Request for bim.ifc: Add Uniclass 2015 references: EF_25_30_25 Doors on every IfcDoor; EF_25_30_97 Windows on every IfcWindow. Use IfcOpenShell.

First a look at what the model holds.

```python
import ifcopenshell

model = ifcopenshell.open("bim.ifc")
print(model.schema)
print("classifications:", [c.Name for c in model.by_type("IfcClassification")])
for ifc_class in ("IfcDoor", "IfcRoof", "IfcStair", "IfcWall", "IfcWindow"):
    print(ifc_class, len(model.by_type(ifc_class)))
```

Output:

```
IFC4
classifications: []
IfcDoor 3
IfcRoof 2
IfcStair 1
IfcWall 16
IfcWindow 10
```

```python
import ifcopenshell
import ifcopenshell.api.classification

model = ifcopenshell.open("bim.ifc")

system = ifcopenshell.api.classification.add_classification(model, classification="Uniclass 2015")

codes = {
    "IfcDoor": ("EF_25_30_25", "Doors"),
    "IfcWindow": ("EF_25_30_97", "Windows"),
}
for ifc_class, (code, name) in codes.items():
    products = model.by_type(ifc_class)
    ifcopenshell.api.classification.add_reference(
        model, products=products, classification=system, identification=code, name=name
    )
    print(code, len(products))

model.write("bim-out.ifc")
```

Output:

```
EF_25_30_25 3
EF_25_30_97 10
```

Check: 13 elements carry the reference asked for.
